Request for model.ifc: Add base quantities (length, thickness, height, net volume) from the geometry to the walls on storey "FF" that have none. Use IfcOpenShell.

First a look at what the model holds.

```python
import ifcopenshell
import ifcopenshell.util.element
import ifcopenshell.util.unit

model = ifcopenshell.open("model.ifc")
print(model.schema)
for unit_type in ("LENGTHUNIT", "AREAUNIT", "VOLUMEUNIT"):
    print(unit_type, ifcopenshell.util.unit.calculate_unit_scale(model, unit_type))
storey = next(s for s in model.by_type("IfcBuildingStorey") if s.Name == "FF")
walls = [e for e in ifcopenshell.util.element.get_decomposition(storey) if e.is_a("IfcWall")]
for e in sorted(walls, key=lambda e: e.id()):
    print(e.id(), e.is_a(), e.Name, list(ifcopenshell.util.element.get_psets(e, qtos_only=True)), sep=" | ")
```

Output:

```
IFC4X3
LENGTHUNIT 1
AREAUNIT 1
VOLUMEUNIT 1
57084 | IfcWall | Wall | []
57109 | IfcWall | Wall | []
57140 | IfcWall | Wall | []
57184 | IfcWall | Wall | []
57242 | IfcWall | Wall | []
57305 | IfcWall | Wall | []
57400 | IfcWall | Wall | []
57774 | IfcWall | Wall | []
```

```python
import ifcopenshell
import ifcopenshell.api.pset
import ifcopenshell.geom
import ifcopenshell.util.element
import ifcopenshell.util.shape
import ifcopenshell.util.unit

model = ifcopenshell.open("model.ifc")
unit_scale = ifcopenshell.util.unit.calculate_unit_scale(model)
volume_scale = ifcopenshell.util.unit.calculate_unit_scale(model, "VOLUMEUNIT")
settings = ifcopenshell.geom.settings()

storey = next(s for s in model.by_type("IfcBuildingStorey") if s.Name == "FF")
walls = [e for e in ifcopenshell.util.element.get_decomposition(storey) if e.is_a("IfcWall")]

for e in sorted(walls, key=lambda e: e.id()):
    if ifcopenshell.util.element.get_psets(e, qtos_only=True, should_inherit=False):
        continue
    # Geometry comes back in metres, in the element's own axes.
    shape = ifcopenshell.geom.create_shape(settings, e)
    values = {
        "Length": ifcopenshell.util.shape.get_x(shape.geometry) / unit_scale,
        "Width": ifcopenshell.util.shape.get_y(shape.geometry) / unit_scale,
        "Height": ifcopenshell.util.shape.get_z(shape.geometry) / unit_scale,
        "NetVolume": ifcopenshell.util.shape.get_volume(shape.geometry) / volume_scale,
    }
    qto = ifcopenshell.api.pset.add_qto(model, product=e, name="Qto_WallBaseQuantities")
    ifcopenshell.api.pset.edit_qto(model, qto=qto, properties=values)
    print(e.id(), {k: round(v, 3) for k, v in values.items()})

model.write("model_edited.ifc")
```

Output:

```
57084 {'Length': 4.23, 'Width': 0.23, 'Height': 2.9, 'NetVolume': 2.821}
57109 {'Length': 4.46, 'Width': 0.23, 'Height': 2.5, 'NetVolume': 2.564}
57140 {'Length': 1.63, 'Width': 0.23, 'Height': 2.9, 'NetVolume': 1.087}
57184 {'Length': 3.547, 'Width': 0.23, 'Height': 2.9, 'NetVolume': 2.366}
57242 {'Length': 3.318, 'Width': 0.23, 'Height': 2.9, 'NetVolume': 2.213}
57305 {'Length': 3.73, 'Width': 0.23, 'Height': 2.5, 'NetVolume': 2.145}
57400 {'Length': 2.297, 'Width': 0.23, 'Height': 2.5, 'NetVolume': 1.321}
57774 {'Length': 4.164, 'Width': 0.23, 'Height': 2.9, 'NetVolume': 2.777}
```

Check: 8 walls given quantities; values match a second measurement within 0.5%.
